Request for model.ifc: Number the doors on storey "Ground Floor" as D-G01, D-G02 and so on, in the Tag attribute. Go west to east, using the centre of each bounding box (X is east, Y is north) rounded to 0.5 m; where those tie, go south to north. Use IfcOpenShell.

First a look at what the model holds.

```python
import ifcopenshell
import ifcopenshell.util.element
import ifcopenshell.util.placement

model = ifcopenshell.open("model.ifc")
print(model.schema)
storey = next(s for s in model.by_type("IfcBuildingStorey") if s.Name == "Ground Floor")
doors = [e for e in ifcopenshell.util.element.get_decomposition(storey) if e.is_a("IfcDoor")]
for e in sorted(doors, key=lambda e: e.id()):
    origin = ifcopenshell.util.placement.get_local_placement(e.ObjectPlacement)[:3, 3]
    print(e.id(), e.Tag, e.Name, origin.round(2) + 0.0, sep=" | ")
```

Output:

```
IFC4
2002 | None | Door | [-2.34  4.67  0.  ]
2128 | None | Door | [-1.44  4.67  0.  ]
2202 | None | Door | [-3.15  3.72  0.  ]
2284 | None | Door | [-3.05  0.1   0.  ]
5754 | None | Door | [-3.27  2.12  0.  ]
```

```python
import ifcopenshell
import ifcopenshell.geom
import ifcopenshell.util.element
import ifcopenshell.util.shape

model = ifcopenshell.open("model.ifc")
settings = ifcopenshell.geom.settings()
settings.set("use-world-coords", True)


def centre(element):
    shape = ifcopenshell.geom.create_shape(settings, element)
    return ifcopenshell.util.shape.get_bbox_centroid(shape.geometry)


storey = next(s for s in model.by_type("IfcBuildingStorey") if s.Name == "Ground Floor")
doors = [e for e in ifcopenshell.util.element.get_decomposition(storey) if e.is_a("IfcDoor")]

# Insertion points can sit at a corner or the storey origin, so sort by the geometry (in metres).
centres = {e: centre(e) for e in doors}
doors.sort(key=lambda e: (round(centres[e][0] / 0.5), centres[e][1]))

for i, e in enumerate(doors, start=1):
    number = f"D-G{i:02d}"
    e.Tag = number
    print(e.id(), number)

model.write("model_edited.ifc")
```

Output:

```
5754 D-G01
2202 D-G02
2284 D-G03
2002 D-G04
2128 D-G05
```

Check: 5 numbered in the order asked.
